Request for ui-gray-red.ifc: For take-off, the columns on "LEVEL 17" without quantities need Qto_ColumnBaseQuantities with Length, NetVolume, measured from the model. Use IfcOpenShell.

First a look at what the model holds.

```python
import ifcopenshell
import ifcopenshell.util.element
import ifcopenshell.util.unit

model = ifcopenshell.open("ui-gray-red.ifc")
print(model.schema)
for unit_type in ("LENGTHUNIT", "AREAUNIT", "VOLUMEUNIT"):
    print(unit_type, ifcopenshell.util.unit.calculate_unit_scale(model, unit_type))
storey = next(s for s in model.by_type("IfcBuildingStorey") if s.Name == "LEVEL 17")
columns = [e for e in ifcopenshell.util.element.get_decomposition(storey) if e.is_a("IfcColumn")]
for e in sorted(columns, key=lambda e: e.id()):
    print(e.id(), e.is_a(), e.Name, list(ifcopenshell.util.element.get_psets(e, qtos_only=True)), sep=" | ")
```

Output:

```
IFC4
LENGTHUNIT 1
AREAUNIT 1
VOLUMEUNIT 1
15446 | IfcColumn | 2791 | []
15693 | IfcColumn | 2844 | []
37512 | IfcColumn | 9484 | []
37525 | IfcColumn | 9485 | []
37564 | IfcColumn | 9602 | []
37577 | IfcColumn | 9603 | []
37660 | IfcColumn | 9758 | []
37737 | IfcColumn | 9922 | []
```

```python
import ifcopenshell
import ifcopenshell.api.pset
import ifcopenshell.geom
import ifcopenshell.util.element
import ifcopenshell.util.shape
import ifcopenshell.util.unit

model = ifcopenshell.open("ui-gray-red.ifc")
unit_scale = ifcopenshell.util.unit.calculate_unit_scale(model)
volume_scale = ifcopenshell.util.unit.calculate_unit_scale(model, "VOLUMEUNIT")
settings = ifcopenshell.geom.settings()

storey = next(s for s in model.by_type("IfcBuildingStorey") if s.Name == "LEVEL 17")
columns = [e for e in ifcopenshell.util.element.get_decomposition(storey) if e.is_a("IfcColumn")]

for e in sorted(columns, key=lambda e: e.id()):
    if ifcopenshell.util.element.get_psets(e, qtos_only=True, should_inherit=False):
        continue
    # Geometry comes back in metres, in the element's own axes.
    shape = ifcopenshell.geom.create_shape(settings, e)
    values = {
        "Length": ifcopenshell.util.shape.get_z(shape.geometry) / unit_scale,
        "NetVolume": ifcopenshell.util.shape.get_volume(shape.geometry) / volume_scale,
    }
    qto = ifcopenshell.api.pset.add_qto(model, product=e, name="Qto_ColumnBaseQuantities")
    ifcopenshell.api.pset.edit_qto(model, qto=qto, properties=values)
    print(e.id(), {k: round(v, 3) for k, v in values.items()})

model.write("ui-gray-red_rev.ifc")
```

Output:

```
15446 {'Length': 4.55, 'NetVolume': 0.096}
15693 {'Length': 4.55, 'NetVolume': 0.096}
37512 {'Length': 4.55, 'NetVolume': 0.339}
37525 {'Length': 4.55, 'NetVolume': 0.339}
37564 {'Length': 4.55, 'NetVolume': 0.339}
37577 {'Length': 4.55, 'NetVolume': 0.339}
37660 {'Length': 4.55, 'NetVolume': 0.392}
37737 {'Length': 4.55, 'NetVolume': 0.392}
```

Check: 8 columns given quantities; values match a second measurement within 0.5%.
